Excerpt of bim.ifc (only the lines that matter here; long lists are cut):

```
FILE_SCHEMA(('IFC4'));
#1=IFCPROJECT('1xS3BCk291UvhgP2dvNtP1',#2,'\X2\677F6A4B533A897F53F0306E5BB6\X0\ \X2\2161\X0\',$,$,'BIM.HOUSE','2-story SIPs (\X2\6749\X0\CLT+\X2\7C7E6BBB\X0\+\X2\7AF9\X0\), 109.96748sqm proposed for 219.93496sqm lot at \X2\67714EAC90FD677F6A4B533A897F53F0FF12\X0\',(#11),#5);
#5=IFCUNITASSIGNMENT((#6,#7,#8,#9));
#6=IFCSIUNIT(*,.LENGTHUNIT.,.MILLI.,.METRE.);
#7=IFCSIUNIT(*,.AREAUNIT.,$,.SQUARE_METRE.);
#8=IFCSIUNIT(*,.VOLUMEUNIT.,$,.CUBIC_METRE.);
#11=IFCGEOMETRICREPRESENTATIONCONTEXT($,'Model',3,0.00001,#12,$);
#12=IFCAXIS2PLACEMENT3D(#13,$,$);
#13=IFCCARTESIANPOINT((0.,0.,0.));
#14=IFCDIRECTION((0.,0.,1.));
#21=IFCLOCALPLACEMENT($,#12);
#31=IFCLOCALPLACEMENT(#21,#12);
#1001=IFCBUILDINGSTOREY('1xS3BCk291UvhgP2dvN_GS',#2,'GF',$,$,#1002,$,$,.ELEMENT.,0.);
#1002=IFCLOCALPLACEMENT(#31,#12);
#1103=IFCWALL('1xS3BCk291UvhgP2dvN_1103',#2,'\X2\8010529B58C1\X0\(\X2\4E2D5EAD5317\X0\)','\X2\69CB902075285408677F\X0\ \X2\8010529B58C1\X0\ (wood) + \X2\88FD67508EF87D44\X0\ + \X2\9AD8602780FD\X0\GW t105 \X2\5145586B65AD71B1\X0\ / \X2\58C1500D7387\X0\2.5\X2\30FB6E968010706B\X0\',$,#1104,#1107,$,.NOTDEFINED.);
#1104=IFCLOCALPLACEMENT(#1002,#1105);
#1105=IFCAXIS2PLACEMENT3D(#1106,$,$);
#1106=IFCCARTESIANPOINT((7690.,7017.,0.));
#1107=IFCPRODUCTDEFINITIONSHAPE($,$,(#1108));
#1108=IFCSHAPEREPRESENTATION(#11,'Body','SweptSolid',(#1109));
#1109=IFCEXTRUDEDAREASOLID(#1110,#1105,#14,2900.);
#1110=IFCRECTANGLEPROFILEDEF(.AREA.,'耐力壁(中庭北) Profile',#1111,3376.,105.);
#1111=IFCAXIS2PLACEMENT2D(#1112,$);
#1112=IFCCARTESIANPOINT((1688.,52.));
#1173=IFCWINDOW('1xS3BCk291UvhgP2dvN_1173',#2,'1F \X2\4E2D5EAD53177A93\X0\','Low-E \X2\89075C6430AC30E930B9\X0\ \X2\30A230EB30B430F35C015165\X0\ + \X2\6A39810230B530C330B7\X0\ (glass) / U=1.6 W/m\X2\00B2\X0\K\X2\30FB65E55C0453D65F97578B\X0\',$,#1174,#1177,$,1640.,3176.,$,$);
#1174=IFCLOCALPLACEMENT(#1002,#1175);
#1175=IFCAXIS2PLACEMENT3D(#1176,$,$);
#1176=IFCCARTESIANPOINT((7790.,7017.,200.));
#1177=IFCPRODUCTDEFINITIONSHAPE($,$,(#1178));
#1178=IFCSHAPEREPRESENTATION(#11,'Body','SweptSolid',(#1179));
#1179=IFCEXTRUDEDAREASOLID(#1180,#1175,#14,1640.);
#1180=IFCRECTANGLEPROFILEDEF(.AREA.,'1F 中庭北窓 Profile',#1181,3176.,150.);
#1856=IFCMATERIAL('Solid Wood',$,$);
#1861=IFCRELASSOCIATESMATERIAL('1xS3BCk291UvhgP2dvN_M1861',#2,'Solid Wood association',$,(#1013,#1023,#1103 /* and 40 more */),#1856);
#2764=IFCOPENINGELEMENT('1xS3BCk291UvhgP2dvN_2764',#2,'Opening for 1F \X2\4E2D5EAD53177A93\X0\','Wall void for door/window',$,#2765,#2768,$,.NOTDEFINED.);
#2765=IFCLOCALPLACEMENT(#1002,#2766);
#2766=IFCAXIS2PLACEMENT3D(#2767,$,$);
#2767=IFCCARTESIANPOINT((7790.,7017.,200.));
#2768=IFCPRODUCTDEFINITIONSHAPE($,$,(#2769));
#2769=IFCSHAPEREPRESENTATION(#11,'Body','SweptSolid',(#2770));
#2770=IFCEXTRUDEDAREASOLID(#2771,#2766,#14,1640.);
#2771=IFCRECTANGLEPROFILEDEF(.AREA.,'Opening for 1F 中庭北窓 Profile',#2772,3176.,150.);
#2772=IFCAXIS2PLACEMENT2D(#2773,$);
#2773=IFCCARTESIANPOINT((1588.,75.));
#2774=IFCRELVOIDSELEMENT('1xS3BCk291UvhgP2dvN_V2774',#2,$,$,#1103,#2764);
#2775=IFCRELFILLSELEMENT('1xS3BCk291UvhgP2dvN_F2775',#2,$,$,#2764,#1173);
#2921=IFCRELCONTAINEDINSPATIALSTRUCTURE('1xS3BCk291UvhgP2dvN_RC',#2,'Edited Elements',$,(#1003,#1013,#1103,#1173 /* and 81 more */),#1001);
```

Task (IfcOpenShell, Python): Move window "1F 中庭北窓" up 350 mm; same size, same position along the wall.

```python
import numpy as np
import ifcopenshell
import ifcopenshell.api.geometry
import ifcopenshell.util.placement
import ifcopenshell.util.unit

model = ifcopenshell.open("bim.ifc")
unit_scale = ifcopenshell.util.unit.calculate_unit_scale(model)

window = model.by_guid("1xS3BCk291UvhgP2dvN_1173")
opening = window.FillsVoids[0].RelatingOpeningElement
dz = 350.0

shift = np.array([0.0, 0.0, dz])
# The window is not placed relative to its opening, so move both.
for product in (opening, window):
    matrix = ifcopenshell.util.placement.get_local_placement(product.ObjectPlacement)
    matrix[:3, 3] += shift
    ifcopenshell.api.geometry.edit_object_placement(model, product=product, matrix=matrix, is_si=False)

print(f"moved by {dz * unit_scale:+.3f} m")

model.write("bim_v2.ifc")
```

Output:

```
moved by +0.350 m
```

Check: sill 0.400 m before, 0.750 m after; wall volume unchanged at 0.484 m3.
